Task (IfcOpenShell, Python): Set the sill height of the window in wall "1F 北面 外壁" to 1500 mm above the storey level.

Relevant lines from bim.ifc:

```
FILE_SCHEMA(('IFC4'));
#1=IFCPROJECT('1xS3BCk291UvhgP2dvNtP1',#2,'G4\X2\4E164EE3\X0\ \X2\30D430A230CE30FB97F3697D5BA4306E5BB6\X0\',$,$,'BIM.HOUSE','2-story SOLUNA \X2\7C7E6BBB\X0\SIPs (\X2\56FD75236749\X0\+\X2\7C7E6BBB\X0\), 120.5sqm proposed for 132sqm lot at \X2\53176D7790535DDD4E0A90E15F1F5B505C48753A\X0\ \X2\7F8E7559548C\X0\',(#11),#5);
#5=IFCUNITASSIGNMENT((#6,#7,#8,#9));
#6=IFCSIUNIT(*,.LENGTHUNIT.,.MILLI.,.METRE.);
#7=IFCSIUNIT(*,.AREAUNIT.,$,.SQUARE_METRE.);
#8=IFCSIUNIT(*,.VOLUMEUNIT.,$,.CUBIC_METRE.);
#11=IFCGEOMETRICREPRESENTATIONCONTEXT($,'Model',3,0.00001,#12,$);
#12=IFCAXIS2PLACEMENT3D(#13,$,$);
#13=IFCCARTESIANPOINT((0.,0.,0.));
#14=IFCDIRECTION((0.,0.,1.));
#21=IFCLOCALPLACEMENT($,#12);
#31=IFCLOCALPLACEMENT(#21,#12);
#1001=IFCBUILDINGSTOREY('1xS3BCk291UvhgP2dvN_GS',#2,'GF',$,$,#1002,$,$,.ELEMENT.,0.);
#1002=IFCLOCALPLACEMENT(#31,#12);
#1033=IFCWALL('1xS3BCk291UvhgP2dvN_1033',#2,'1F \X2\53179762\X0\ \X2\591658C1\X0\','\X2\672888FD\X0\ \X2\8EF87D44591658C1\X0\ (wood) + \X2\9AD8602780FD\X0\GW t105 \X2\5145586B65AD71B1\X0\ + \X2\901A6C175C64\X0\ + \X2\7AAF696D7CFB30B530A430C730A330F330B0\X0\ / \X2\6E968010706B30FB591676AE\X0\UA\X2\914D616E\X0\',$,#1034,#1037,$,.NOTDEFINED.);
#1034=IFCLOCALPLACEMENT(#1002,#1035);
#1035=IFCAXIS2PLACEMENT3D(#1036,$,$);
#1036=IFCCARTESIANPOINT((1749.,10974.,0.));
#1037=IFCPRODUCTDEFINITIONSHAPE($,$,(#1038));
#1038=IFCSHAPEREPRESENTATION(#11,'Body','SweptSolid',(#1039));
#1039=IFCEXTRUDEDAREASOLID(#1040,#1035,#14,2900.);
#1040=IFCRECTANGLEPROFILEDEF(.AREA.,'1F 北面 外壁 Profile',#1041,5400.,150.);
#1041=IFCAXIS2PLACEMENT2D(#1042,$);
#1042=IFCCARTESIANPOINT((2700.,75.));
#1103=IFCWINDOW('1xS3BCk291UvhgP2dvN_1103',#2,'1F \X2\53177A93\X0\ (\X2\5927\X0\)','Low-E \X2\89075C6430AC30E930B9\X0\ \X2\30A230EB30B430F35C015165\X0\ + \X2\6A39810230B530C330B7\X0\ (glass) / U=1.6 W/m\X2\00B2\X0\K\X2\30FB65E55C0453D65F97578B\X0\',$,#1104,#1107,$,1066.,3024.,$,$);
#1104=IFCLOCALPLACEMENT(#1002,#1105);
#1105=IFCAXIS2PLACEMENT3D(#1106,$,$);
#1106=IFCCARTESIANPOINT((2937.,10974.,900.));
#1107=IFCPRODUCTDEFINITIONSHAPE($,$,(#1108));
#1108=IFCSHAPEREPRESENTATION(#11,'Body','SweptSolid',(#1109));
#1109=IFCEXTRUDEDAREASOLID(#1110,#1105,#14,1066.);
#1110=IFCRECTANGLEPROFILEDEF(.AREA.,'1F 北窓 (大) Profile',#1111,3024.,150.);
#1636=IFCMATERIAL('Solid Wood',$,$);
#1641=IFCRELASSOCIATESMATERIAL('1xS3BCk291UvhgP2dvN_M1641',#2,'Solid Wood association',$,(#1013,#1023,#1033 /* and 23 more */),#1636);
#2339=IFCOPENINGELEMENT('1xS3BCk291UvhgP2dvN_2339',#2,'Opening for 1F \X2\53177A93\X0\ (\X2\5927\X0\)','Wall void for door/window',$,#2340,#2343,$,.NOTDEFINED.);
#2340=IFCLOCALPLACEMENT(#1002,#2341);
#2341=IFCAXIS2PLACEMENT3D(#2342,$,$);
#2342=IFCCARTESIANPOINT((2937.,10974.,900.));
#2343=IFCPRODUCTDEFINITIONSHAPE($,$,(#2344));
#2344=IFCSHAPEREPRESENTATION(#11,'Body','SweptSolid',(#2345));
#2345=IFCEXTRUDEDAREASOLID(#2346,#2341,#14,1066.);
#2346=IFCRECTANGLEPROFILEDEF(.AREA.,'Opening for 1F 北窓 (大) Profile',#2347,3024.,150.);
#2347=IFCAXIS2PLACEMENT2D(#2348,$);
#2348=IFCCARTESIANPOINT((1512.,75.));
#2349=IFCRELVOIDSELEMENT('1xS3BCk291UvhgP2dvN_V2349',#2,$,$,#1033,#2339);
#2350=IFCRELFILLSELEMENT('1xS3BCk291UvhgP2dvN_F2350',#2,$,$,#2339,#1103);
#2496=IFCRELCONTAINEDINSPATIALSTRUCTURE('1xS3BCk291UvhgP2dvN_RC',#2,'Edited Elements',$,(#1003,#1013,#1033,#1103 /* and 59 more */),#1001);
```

```python
import numpy as np
import ifcopenshell
import ifcopenshell.api.geometry
import ifcopenshell.geom
import ifcopenshell.util.element
import ifcopenshell.util.placement
import ifcopenshell.util.shape
import ifcopenshell.util.unit

model = ifcopenshell.open("bim.ifc")
unit_scale = ifcopenshell.util.unit.calculate_unit_scale(model)

window = model.by_guid("1xS3BCk291UvhgP2dvN_1103")
opening = window.FillsVoids[0].RelatingOpeningElement
storey = ifcopenshell.util.element.get_container(window, ifc_class="IfcBuildingStorey")
level = ifcopenshell.util.placement.get_local_placement(storey.ObjectPlacement)[2, 3]

# The opening's origin need not be at the sill, so measure its lowest point.
shape = ifcopenshell.geom.create_shape(ifcopenshell.geom.settings(), opening)
bottom = ifcopenshell.util.shape.get_shape_bottom_elevation(shape, shape.geometry) / unit_scale
dz = level + 1.5 / unit_scale - bottom

shift = np.array([0.0, 0.0, dz])
# The window is not placed relative to its opening, so move both.
for product in (opening, window):
    matrix = ifcopenshell.util.placement.get_local_placement(product.ObjectPlacement)
    matrix[:3, 3] += shift
    ifcopenshell.api.geometry.edit_object_placement(model, product=product, matrix=matrix, is_si=False)

print(f"moved by {dz * unit_scale:+.3f} m")

model.write("bim_v2.ifc")
```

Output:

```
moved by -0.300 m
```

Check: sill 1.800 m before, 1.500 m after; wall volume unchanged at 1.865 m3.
